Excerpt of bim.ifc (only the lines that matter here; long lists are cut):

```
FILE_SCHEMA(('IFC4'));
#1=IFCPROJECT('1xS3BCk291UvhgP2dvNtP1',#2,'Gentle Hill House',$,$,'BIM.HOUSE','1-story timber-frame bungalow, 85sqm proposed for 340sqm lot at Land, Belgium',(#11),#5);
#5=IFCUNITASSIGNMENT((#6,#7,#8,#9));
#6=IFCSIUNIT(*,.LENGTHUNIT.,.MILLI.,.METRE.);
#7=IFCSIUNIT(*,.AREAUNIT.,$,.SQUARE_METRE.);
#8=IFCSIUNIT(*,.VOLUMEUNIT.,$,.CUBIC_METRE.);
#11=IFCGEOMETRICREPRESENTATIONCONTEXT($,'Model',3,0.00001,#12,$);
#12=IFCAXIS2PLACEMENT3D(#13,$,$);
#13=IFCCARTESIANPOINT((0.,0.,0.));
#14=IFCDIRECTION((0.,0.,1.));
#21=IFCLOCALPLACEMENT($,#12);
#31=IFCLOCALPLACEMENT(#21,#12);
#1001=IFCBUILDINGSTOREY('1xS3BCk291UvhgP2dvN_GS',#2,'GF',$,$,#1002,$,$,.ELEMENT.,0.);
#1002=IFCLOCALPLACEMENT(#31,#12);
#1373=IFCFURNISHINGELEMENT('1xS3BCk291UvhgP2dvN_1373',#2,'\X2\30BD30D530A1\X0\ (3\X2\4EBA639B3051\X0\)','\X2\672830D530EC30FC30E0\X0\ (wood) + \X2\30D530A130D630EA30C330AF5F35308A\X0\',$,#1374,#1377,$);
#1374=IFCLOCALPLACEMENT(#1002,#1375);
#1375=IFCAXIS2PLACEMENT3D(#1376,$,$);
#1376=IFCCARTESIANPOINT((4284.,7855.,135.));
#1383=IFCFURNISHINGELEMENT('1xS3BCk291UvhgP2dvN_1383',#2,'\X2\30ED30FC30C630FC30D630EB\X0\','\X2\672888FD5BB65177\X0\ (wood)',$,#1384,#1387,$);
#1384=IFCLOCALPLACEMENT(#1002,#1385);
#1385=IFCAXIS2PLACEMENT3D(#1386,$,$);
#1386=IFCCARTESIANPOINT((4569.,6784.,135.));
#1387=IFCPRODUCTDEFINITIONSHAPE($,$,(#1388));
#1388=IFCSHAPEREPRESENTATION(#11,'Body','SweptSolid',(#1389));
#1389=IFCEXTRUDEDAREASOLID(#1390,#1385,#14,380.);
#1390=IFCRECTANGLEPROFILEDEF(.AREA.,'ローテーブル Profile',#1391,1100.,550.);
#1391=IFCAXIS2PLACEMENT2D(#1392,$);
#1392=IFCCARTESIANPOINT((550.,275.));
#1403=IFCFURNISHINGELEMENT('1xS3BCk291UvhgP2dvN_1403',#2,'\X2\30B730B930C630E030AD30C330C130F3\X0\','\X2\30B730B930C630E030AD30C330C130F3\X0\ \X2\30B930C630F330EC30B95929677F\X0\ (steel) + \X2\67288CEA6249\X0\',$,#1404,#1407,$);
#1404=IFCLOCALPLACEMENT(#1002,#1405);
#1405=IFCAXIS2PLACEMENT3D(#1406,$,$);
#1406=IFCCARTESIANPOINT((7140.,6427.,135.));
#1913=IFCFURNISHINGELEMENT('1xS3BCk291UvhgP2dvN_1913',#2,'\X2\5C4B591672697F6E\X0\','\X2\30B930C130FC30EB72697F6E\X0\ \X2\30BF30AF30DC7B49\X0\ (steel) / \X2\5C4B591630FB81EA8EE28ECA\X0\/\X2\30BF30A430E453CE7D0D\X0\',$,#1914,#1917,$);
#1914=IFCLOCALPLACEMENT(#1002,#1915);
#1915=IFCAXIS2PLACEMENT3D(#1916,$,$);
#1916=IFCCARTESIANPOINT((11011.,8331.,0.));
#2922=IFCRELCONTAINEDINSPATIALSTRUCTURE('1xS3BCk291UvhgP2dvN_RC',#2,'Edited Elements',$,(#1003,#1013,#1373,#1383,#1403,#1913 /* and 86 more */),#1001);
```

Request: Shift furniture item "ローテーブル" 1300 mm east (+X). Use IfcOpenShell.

```python
import ifcopenshell
import ifcopenshell.api.geometry
import ifcopenshell.util.placement
import ifcopenshell.util.unit

model = ifcopenshell.open("bim.ifc")
unit_scale = ifcopenshell.util.unit.calculate_unit_scale(model)

item = model.by_guid("1xS3BCk291UvhgP2dvN_1383")
matrix = ifcopenshell.util.placement.get_local_placement(item.ObjectPlacement)
matrix[0, 3] += 1.3 / unit_scale
ifcopenshell.api.geometry.edit_object_placement(model, product=item, matrix=matrix, is_si=False)

print(ifcopenshell.util.placement.get_local_placement(item.ObjectPlacement).round(3) + 0.0)

model.write("bim-out.ifc")
```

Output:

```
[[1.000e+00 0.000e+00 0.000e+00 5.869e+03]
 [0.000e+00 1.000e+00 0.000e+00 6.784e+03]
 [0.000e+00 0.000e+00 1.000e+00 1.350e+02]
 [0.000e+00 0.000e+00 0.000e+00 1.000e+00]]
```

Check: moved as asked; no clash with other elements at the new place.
